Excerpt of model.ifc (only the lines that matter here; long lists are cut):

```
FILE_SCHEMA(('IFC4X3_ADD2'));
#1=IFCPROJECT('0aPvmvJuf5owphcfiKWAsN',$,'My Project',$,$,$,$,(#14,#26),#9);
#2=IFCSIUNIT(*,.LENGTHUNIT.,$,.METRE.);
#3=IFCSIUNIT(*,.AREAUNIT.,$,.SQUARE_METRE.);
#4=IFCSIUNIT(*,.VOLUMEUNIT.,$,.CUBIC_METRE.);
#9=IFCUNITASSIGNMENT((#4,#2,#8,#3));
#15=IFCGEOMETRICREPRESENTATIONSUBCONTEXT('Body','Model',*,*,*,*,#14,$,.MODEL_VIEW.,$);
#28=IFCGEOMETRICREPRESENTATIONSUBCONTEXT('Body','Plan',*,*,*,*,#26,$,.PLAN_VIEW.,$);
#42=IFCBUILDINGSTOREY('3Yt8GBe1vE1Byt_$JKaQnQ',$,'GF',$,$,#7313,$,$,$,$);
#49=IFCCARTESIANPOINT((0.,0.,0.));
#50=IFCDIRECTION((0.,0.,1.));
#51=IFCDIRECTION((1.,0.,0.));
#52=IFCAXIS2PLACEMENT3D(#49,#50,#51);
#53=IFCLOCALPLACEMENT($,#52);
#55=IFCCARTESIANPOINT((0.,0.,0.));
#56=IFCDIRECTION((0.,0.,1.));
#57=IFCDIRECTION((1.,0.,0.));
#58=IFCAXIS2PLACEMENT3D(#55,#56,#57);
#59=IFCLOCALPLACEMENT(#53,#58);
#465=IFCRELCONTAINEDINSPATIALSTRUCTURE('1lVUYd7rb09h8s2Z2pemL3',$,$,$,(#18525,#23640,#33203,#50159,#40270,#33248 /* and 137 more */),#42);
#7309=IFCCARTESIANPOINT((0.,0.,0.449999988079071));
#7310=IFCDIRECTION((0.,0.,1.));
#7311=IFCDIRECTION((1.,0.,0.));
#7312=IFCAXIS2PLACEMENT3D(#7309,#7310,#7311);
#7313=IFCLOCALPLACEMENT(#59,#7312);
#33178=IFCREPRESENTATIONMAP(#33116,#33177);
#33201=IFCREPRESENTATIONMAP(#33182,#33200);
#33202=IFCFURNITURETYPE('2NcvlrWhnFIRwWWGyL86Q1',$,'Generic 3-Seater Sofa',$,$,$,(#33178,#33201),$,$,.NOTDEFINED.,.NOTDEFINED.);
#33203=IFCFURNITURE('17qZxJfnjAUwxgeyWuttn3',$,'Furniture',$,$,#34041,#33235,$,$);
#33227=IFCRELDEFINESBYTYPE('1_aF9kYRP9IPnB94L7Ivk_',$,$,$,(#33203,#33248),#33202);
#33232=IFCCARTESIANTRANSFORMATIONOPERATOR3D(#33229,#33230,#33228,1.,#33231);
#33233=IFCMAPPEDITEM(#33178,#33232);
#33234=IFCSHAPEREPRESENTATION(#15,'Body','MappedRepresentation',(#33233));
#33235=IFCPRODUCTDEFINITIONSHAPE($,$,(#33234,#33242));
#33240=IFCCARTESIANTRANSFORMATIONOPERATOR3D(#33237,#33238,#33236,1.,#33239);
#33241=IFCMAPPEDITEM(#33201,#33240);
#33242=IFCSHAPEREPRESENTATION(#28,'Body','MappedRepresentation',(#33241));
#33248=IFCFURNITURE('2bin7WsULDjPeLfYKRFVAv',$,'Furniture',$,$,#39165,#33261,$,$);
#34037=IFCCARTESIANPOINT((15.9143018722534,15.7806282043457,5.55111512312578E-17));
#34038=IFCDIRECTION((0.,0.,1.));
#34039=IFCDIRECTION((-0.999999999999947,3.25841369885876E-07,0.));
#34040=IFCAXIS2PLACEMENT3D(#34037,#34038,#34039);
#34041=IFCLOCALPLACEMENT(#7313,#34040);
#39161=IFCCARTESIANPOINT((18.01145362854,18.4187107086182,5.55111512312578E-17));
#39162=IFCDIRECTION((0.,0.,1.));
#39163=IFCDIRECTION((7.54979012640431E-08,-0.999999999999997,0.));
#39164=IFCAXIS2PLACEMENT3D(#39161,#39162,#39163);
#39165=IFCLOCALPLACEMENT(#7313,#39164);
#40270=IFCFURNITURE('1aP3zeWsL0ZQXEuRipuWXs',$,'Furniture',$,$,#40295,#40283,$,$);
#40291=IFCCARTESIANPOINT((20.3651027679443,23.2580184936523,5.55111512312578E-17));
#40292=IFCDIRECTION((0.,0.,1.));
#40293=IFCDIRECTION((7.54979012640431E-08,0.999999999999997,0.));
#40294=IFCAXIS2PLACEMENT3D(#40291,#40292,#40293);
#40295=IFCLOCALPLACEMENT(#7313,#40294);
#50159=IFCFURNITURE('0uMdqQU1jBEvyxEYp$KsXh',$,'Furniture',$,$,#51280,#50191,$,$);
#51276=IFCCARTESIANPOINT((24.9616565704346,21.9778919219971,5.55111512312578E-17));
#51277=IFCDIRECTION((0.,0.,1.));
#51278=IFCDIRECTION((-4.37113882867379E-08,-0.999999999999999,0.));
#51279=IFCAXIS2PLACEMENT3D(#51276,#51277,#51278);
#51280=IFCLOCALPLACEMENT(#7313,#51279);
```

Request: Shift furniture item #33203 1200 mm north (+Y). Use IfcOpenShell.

```python
import ifcopenshell
import ifcopenshell.api.geometry
import ifcopenshell.util.placement

model = ifcopenshell.open("model.ifc")

item = model.by_id(33203)
matrix = ifcopenshell.util.placement.get_local_placement(item.ObjectPlacement)
matrix[1, 3] += 1.2
ifcopenshell.api.geometry.edit_object_placement(model, product=item, matrix=matrix, is_si=False)

print(ifcopenshell.util.placement.get_local_placement(item.ObjectPlacement).round(3) + 0.0)

model.write("model_updated.ifc")
```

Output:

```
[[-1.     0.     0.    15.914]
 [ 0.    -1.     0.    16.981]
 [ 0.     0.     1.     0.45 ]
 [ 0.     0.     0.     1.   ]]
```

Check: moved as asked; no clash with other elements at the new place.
